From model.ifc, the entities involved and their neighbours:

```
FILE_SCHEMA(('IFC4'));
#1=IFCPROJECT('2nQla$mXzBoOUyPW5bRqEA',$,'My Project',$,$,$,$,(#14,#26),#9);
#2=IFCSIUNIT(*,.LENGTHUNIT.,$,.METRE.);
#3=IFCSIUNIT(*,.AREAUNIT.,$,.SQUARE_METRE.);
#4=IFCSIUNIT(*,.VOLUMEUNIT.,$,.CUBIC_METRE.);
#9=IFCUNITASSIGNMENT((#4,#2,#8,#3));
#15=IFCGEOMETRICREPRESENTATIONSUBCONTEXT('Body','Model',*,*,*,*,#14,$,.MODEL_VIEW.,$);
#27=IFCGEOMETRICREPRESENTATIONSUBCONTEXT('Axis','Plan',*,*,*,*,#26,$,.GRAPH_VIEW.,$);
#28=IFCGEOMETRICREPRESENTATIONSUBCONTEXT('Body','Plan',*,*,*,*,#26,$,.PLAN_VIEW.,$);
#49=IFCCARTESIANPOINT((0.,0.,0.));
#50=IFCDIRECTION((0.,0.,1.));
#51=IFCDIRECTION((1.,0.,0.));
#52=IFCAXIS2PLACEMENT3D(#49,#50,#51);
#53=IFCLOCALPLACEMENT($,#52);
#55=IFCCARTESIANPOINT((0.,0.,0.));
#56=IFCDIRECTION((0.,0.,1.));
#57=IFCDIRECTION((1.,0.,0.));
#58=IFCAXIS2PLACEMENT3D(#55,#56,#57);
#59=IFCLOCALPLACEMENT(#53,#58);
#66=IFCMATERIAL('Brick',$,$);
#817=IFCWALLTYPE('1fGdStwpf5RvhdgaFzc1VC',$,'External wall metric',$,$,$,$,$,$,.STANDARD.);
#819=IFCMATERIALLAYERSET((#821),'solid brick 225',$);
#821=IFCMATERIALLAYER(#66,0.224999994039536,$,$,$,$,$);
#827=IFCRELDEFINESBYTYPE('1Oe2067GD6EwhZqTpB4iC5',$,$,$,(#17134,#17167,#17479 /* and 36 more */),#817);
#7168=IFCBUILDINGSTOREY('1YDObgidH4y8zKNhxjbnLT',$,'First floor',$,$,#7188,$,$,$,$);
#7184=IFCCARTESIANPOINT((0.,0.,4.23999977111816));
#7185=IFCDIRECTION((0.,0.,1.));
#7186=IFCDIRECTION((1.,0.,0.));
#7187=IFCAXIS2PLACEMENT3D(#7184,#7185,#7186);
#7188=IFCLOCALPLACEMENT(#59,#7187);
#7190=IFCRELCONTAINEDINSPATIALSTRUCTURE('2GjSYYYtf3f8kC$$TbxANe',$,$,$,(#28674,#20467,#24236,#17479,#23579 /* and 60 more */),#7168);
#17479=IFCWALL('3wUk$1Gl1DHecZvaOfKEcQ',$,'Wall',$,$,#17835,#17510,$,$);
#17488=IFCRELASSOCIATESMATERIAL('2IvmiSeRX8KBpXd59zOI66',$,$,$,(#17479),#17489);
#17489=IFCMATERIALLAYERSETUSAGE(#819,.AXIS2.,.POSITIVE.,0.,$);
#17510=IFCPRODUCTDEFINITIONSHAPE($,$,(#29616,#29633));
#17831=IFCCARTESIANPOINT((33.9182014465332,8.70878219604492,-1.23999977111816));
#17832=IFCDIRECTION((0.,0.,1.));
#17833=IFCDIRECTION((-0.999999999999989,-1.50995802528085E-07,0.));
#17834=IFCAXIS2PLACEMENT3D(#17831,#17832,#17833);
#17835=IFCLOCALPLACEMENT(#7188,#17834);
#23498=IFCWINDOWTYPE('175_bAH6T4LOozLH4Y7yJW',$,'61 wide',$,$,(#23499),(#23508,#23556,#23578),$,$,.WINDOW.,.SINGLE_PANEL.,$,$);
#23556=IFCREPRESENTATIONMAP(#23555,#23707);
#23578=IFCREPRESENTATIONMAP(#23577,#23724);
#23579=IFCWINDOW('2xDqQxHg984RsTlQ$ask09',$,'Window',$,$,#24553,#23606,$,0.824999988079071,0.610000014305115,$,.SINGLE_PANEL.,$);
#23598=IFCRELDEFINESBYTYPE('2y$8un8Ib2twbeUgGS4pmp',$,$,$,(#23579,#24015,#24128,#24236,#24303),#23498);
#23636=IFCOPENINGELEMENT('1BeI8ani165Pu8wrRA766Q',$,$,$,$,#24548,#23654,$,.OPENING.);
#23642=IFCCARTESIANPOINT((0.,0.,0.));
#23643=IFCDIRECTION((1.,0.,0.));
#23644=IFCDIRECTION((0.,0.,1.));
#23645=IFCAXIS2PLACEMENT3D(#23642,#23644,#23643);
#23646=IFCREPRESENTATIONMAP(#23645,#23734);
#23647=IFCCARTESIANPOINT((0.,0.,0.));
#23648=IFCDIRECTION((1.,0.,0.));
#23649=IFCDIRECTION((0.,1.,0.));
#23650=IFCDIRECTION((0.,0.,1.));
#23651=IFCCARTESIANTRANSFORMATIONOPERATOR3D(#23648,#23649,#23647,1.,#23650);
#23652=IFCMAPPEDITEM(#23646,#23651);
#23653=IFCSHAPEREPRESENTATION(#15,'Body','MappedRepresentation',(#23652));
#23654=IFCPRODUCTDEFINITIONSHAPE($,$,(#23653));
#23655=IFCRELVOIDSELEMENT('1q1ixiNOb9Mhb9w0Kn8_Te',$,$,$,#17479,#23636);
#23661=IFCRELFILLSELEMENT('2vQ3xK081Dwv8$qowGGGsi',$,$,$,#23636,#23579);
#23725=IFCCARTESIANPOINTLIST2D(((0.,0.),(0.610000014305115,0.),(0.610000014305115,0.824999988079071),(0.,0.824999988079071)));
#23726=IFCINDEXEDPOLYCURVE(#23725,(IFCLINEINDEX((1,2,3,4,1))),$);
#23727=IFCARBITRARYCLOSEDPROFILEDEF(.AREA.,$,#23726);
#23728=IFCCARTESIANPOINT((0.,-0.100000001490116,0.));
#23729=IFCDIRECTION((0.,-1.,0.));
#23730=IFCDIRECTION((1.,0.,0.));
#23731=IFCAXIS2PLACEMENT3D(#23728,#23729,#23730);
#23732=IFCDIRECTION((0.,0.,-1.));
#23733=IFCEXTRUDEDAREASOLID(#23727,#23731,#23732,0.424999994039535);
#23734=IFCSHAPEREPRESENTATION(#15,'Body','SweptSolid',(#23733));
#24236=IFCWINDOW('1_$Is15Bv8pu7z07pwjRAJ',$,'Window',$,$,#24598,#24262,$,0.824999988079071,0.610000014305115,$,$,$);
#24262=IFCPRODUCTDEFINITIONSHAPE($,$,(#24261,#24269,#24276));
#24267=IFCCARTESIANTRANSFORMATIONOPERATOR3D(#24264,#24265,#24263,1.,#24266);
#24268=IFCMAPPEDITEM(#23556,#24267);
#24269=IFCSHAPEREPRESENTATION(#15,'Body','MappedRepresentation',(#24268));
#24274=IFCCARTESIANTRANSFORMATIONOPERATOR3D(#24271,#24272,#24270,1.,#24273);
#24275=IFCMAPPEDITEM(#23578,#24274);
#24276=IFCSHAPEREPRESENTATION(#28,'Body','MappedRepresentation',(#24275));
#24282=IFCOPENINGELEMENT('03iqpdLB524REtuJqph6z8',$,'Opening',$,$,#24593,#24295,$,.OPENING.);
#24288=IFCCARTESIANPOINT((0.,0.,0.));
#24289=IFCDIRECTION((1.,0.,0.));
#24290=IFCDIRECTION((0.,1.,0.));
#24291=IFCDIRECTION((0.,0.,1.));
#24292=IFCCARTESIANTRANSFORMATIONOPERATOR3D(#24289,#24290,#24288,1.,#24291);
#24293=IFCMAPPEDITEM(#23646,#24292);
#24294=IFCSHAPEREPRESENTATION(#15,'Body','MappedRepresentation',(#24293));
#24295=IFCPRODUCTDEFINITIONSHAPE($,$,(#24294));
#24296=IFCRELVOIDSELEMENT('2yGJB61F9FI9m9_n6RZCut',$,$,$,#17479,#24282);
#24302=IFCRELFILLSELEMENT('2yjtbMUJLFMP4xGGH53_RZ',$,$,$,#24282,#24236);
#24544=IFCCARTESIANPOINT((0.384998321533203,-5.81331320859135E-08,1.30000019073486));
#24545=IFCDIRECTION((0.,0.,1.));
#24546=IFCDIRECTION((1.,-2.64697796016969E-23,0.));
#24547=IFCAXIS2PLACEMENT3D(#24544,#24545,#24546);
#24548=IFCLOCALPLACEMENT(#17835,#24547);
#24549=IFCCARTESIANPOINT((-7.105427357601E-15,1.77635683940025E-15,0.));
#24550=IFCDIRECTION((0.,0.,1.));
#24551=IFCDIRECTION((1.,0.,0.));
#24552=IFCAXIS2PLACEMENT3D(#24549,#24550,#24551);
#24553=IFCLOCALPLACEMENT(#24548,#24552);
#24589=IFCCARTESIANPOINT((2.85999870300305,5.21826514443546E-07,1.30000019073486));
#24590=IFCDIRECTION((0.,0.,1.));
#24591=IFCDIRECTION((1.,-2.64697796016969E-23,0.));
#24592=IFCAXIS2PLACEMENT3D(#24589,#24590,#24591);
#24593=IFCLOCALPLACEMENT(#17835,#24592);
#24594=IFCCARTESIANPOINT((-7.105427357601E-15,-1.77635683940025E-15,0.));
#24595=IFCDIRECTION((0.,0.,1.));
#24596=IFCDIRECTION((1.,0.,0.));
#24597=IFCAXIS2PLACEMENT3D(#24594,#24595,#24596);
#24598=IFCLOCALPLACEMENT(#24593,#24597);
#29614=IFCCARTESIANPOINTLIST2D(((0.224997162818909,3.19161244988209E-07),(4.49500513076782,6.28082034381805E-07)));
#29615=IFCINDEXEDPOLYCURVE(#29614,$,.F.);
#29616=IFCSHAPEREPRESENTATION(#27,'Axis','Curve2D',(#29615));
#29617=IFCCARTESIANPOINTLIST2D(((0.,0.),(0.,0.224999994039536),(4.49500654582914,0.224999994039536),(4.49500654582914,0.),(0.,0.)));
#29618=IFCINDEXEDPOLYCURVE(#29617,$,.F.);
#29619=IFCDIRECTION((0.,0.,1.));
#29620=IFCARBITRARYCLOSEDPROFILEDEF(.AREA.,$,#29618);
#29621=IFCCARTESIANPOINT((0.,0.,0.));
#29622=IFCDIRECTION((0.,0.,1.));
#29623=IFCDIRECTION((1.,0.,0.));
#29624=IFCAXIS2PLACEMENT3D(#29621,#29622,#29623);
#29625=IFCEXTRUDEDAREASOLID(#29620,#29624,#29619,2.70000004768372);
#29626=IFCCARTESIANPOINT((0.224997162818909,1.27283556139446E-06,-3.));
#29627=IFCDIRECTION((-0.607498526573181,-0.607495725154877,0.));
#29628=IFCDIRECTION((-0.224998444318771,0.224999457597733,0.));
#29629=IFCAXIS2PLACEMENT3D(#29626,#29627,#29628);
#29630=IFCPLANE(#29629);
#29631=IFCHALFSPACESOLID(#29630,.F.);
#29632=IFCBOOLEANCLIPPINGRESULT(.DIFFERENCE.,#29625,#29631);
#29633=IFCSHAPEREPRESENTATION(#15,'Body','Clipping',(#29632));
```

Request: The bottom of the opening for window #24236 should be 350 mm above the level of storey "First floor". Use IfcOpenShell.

```python
import numpy as np
import ifcopenshell
import ifcopenshell.api.geometry
import ifcopenshell.geom
import ifcopenshell.util.element
import ifcopenshell.util.placement
import ifcopenshell.util.shape
import ifcopenshell.util.unit

model = ifcopenshell.open("model.ifc")
unit_scale = ifcopenshell.util.unit.calculate_unit_scale(model)

window = model.by_guid("1_$Is15Bv8pu7z07pwjRAJ")
opening = window.FillsVoids[0].RelatingOpeningElement
storey = ifcopenshell.util.element.get_container(window, ifc_class="IfcBuildingStorey")
level = ifcopenshell.util.placement.get_local_placement(storey.ObjectPlacement)[2, 3]

# The opening's origin need not be at the sill, so measure its lowest point.
shape = ifcopenshell.geom.create_shape(ifcopenshell.geom.settings(), opening)
bottom = ifcopenshell.util.shape.get_shape_bottom_elevation(shape, shape.geometry) / unit_scale
dz = level + 0.35 - bottom

shift = np.array([0.0, 0.0, dz])
# The window is placed relative to its opening, so it follows when the opening moves.
matrix = ifcopenshell.util.placement.get_local_placement(opening.ObjectPlacement)
matrix[:3, 3] += shift
ifcopenshell.api.geometry.edit_object_placement(
    model, product=opening, matrix=matrix, is_si=False, should_transform_children=True
)

print(f"moved by {dz * unit_scale:+.3f} m")

model.write("model_v2.ifc")
```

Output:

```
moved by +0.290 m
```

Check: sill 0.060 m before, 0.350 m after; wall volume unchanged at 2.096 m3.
